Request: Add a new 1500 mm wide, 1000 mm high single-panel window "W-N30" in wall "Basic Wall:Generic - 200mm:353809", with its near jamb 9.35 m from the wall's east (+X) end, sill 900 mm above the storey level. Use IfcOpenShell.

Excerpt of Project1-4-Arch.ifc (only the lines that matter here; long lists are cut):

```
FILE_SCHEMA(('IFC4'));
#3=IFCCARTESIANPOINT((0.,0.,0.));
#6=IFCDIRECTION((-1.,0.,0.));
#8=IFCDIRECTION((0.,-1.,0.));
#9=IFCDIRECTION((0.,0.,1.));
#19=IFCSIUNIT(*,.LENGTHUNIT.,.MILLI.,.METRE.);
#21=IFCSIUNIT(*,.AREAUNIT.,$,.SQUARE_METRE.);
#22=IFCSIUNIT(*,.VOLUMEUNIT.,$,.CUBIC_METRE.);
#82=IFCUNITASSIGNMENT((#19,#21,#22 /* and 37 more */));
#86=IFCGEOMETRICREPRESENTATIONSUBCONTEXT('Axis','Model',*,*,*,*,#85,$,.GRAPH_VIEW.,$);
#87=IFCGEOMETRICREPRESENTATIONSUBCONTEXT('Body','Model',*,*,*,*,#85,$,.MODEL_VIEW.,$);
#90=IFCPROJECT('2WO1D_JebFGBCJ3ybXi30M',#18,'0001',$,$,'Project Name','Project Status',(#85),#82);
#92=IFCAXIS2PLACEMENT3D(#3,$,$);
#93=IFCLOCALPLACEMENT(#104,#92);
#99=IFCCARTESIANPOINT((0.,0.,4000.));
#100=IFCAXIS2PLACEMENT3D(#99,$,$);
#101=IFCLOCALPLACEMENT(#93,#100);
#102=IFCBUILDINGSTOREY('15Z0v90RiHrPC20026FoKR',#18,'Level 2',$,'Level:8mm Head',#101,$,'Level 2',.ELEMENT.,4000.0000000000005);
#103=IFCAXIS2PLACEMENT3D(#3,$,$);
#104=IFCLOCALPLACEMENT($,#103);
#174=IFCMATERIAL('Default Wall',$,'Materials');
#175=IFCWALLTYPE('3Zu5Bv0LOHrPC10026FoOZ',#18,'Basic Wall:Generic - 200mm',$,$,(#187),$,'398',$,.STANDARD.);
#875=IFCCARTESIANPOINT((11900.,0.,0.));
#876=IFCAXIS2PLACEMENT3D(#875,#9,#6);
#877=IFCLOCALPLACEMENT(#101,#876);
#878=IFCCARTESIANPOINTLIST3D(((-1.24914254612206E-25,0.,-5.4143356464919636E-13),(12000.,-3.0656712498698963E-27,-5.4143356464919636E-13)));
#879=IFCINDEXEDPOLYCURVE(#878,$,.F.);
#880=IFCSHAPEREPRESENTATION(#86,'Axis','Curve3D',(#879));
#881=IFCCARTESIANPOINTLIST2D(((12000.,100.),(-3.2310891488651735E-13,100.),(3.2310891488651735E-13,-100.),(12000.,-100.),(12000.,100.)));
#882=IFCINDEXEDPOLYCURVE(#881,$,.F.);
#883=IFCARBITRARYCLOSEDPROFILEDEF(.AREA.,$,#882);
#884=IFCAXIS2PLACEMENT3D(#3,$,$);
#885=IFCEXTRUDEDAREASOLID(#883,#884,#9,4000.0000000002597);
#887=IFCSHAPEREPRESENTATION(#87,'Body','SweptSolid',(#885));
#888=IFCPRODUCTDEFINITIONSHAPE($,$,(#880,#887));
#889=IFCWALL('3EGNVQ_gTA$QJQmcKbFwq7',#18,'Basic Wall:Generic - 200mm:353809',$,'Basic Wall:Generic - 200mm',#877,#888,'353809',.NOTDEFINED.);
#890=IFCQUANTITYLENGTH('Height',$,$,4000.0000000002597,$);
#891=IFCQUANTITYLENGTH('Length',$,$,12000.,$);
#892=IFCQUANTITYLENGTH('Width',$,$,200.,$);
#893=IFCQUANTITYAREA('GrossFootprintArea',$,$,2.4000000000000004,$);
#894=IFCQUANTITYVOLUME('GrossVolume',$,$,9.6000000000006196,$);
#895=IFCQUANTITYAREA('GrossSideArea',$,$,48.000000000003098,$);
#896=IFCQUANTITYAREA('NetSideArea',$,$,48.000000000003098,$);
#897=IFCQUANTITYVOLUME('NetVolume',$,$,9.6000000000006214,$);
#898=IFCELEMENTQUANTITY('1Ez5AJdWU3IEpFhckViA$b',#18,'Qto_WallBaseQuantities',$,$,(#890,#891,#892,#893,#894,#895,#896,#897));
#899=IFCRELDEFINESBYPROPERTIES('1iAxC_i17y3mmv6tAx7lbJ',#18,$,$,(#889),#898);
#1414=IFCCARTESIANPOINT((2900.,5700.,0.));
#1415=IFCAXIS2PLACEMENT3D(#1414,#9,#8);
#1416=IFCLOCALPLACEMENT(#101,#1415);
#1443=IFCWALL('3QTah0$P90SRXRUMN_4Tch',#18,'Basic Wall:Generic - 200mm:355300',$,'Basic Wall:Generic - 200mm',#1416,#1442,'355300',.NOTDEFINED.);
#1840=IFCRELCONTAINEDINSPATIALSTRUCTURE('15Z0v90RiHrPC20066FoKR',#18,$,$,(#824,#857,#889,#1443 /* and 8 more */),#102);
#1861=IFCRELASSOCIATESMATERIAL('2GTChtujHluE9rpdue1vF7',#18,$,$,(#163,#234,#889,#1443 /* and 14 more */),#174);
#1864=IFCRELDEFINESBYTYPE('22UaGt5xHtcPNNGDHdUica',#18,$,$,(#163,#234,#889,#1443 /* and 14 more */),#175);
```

```python
import numpy as np
import ifcopenshell
import ifcopenshell.api.feature
import ifcopenshell.api.geometry
import ifcopenshell.api.pset
import ifcopenshell.api.root
import ifcopenshell.api.spatial
import ifcopenshell.geom
import ifcopenshell.util.element
import ifcopenshell.util.placement
import ifcopenshell.util.representation
import ifcopenshell.util.shape
import ifcopenshell.util.unit

model = ifcopenshell.open("Project1-4-Arch.ifc")
unit_scale = ifcopenshell.util.unit.calculate_unit_scale(model)
area_scale = ifcopenshell.util.unit.calculate_unit_scale(model, "AREAUNIT")
volume_scale = ifcopenshell.util.unit.calculate_unit_scale(model, "VOLUMEUNIT")
settings = ifcopenshell.geom.settings()


def volume(element):
    """Net volume in cubic metres, openings subtracted."""
    shape = ifcopenshell.geom.create_shape(settings, element)
    return ifcopenshell.util.shape.get_volume(shape.geometry)


wall = model.by_id(889)
storey = ifcopenshell.util.element.get_container(wall, ifc_class="IfcBuildingStorey")
context = ifcopenshell.util.representation.get_context(model, "Model", "Body", "MODEL_VIEW")
before = volume(wall)

width, height, from_end, sill = 1.5, 1, 9.35, 0.9  # metres

# The wall runs along its own X axis, and the end named is its -X end.
wall_shape = ifcopenshell.geom.create_shape(settings, wall)
x, y, z = ifcopenshell.util.shape.get_vertices(wall_shape.geometry).T
start = x.min() + from_end
face, thickness = float(y.min()), float(y.max() - y.min())
wall_matrix = ifcopenshell.util.placement.get_local_placement(wall.ObjectPlacement)
level = ifcopenshell.util.placement.get_local_placement(storey.ObjectPlacement)[2, 3]


def in_wall(x, y):
    """Placement at x, y metres in the wall's axes, at sill height."""
    matrix = wall_matrix.copy()
    matrix[:, 3] = wall_matrix @ np.array([x / unit_scale, y / unit_scale, 0.0, 1.0])
    matrix[2, 3] = level + sill / unit_scale
    return matrix


# Opening: a box that overshoots both wall faces by 50 mm.
opening = ifcopenshell.api.root.create_entity(model, ifc_class="IfcOpeningElement", predefined_type="OPENING")
box = ifcopenshell.api.geometry.add_wall_representation(
    model, context=context, length=width, height=height, thickness=thickness + 0.1
)
ifcopenshell.api.geometry.assign_representation(model, product=opening, representation=box)
ifcopenshell.api.geometry.edit_object_placement(model, product=opening, matrix=in_wall(start, face - 0.05), is_si=False)
ifcopenshell.api.feature.add_feature(model, feature=opening, element=wall)

window = ifcopenshell.api.root.create_entity(model, ifc_class="IfcWindow", name="W-N30", predefined_type="WINDOW")
window.OverallWidth, window.OverallHeight = width / unit_scale, height / unit_scale
window.PartitioningType = "SINGLE_PANEL"
body = ifcopenshell.api.geometry.add_window_representation(
    model,
    context=context,
    overall_width=window.OverallWidth,
    overall_height=window.OverallHeight,
    partition_type="SINGLE_PANEL",
)
ifcopenshell.api.geometry.assign_representation(model, product=window, representation=body)
ifcopenshell.api.spatial.assign_container(model, products=[window], relating_structure=storey)
ifcopenshell.api.feature.add_filling(model, opening=opening, element=window)

# Centre the window in the wall's thickness.
ifcopenshell.api.geometry.edit_object_placement(model, product=window, matrix=in_wall(start, face), is_si=False)
window_shape = ifcopenshell.geom.create_shape(settings, window)
depth = ifcopenshell.util.shape.get_vertices(window_shape.geometry)[:, 1]
offset = face + thickness / 2 - (depth.min() + depth.max()) / 2
ifcopenshell.api.geometry.edit_object_placement(model, product=window, matrix=in_wall(start, offset), is_si=False)

after = volume(wall)

# Update the wall's stored quantities.
qto = model.by_id(ifcopenshell.util.element.get_pset(wall, "Qto_WallBaseQuantities", should_inherit=False)["id"])
ifcopenshell.api.pset.edit_qto(model, qto=qto, properties={
    "NetSideArea": after / thickness / area_scale,
    "NetVolume": after / volume_scale,
})

print(f"wall volume {before:.3f} -> {after:.3f} m3")

model.write("Project1-4-Arch_edited.ifc")
```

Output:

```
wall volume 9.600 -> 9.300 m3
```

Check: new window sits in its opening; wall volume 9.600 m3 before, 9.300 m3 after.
